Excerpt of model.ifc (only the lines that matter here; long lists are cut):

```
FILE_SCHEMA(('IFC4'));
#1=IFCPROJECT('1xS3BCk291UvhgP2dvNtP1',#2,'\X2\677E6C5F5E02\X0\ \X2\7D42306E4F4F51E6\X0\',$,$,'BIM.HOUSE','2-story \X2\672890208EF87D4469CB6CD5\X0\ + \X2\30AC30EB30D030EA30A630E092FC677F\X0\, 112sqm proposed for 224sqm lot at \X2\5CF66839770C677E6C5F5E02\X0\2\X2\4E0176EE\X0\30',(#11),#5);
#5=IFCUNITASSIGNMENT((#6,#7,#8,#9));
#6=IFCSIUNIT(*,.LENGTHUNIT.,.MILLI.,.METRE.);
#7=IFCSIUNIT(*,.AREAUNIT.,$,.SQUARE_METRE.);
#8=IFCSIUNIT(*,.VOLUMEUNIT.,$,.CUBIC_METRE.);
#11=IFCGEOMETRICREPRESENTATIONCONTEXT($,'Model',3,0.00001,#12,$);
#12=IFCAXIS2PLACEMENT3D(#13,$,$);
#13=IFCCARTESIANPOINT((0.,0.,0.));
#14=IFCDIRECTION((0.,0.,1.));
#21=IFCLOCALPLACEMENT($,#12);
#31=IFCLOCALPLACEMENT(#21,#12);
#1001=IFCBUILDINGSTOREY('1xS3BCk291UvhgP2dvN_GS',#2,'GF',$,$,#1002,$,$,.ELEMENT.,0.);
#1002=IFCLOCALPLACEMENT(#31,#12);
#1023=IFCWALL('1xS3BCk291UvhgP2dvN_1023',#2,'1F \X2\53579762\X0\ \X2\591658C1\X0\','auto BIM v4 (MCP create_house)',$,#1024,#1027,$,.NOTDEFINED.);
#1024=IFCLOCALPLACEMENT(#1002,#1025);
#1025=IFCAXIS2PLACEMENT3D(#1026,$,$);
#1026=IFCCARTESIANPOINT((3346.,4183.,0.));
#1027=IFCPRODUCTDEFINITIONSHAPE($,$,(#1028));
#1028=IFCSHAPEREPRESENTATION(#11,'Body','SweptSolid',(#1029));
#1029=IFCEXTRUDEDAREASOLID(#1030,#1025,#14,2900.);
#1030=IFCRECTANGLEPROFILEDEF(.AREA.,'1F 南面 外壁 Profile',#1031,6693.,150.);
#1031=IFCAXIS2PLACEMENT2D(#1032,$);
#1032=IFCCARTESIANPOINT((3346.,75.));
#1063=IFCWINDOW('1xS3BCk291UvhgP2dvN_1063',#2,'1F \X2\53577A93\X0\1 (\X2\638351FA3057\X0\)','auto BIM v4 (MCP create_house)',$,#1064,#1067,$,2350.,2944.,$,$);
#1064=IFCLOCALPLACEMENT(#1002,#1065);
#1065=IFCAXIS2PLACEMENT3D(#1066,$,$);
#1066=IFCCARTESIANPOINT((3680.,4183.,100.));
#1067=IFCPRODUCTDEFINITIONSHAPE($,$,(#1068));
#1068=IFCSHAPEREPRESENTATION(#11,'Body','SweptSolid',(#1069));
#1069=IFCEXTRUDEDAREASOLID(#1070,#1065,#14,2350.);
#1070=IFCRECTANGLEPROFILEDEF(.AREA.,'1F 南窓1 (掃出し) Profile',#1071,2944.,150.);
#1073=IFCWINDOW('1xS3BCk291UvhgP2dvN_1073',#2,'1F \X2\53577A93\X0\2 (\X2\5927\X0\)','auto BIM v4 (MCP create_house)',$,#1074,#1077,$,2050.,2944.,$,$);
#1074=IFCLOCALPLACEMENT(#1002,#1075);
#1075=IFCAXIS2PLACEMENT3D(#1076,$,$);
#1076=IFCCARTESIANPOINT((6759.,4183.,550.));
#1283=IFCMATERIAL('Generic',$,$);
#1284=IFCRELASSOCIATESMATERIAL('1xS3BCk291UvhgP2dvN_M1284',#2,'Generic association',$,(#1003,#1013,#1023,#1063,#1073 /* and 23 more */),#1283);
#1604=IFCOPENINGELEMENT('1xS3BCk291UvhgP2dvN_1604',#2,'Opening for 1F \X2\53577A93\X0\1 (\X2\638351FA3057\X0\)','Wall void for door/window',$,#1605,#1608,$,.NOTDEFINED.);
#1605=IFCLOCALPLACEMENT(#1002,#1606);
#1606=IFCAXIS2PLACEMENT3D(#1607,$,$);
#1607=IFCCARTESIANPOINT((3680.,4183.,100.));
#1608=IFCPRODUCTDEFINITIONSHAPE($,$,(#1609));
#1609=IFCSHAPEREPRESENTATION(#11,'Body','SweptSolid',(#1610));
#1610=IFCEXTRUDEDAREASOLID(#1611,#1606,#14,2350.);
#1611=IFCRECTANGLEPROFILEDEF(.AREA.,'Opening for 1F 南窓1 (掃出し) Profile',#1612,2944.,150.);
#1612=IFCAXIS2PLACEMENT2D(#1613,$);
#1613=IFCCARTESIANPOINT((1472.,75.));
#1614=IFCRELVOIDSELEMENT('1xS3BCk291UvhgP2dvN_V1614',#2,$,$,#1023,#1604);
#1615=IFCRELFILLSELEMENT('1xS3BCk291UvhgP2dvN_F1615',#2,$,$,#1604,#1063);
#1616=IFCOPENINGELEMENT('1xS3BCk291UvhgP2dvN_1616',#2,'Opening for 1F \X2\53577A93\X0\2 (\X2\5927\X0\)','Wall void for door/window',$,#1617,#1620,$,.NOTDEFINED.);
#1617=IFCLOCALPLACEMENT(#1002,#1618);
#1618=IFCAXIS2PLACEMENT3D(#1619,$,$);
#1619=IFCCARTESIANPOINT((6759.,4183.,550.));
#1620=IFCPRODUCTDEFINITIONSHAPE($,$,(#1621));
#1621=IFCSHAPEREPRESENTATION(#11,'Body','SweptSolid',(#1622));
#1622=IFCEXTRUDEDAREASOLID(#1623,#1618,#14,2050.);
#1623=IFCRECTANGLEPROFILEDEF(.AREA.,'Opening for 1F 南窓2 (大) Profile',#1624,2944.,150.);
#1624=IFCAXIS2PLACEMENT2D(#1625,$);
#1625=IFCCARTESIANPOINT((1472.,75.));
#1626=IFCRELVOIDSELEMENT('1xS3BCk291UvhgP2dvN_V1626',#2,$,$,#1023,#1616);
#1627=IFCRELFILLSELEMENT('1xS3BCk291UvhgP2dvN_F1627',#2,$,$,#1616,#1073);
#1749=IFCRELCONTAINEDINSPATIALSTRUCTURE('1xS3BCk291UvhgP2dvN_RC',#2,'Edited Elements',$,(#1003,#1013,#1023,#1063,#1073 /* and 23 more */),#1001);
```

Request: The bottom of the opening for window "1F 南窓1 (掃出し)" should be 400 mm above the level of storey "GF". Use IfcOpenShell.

```python
import numpy as np
import ifcopenshell
import ifcopenshell.api.geometry
import ifcopenshell.geom
import ifcopenshell.util.element
import ifcopenshell.util.placement
import ifcopenshell.util.shape
import ifcopenshell.util.unit

model = ifcopenshell.open("model.ifc")
unit_scale = ifcopenshell.util.unit.calculate_unit_scale(model)

window = model.by_guid("1xS3BCk291UvhgP2dvN_1063")
opening = window.FillsVoids[0].RelatingOpeningElement
storey = ifcopenshell.util.element.get_container(window, ifc_class="IfcBuildingStorey")
level = ifcopenshell.util.placement.get_local_placement(storey.ObjectPlacement)[2, 3]

# The opening's origin need not be at the sill, so measure its lowest point.
shape = ifcopenshell.geom.create_shape(ifcopenshell.geom.settings(), opening)
bottom = ifcopenshell.util.shape.get_shape_bottom_elevation(shape, shape.geometry) / unit_scale
dz = level + 400.0 - bottom

shift = np.array([0.0, 0.0, dz])
# The window is not placed relative to its opening, so move both.
for product in (opening, window):
    matrix = ifcopenshell.util.placement.get_local_placement(product.ObjectPlacement)
    matrix[:3, 3] += shift
    ifcopenshell.api.geometry.edit_object_placement(model, product=product, matrix=matrix, is_si=False)

print(f"moved by {dz * unit_scale:+.3f} m")

model.write("model-out.ifc")
```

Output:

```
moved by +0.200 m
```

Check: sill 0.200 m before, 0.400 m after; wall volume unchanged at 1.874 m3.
